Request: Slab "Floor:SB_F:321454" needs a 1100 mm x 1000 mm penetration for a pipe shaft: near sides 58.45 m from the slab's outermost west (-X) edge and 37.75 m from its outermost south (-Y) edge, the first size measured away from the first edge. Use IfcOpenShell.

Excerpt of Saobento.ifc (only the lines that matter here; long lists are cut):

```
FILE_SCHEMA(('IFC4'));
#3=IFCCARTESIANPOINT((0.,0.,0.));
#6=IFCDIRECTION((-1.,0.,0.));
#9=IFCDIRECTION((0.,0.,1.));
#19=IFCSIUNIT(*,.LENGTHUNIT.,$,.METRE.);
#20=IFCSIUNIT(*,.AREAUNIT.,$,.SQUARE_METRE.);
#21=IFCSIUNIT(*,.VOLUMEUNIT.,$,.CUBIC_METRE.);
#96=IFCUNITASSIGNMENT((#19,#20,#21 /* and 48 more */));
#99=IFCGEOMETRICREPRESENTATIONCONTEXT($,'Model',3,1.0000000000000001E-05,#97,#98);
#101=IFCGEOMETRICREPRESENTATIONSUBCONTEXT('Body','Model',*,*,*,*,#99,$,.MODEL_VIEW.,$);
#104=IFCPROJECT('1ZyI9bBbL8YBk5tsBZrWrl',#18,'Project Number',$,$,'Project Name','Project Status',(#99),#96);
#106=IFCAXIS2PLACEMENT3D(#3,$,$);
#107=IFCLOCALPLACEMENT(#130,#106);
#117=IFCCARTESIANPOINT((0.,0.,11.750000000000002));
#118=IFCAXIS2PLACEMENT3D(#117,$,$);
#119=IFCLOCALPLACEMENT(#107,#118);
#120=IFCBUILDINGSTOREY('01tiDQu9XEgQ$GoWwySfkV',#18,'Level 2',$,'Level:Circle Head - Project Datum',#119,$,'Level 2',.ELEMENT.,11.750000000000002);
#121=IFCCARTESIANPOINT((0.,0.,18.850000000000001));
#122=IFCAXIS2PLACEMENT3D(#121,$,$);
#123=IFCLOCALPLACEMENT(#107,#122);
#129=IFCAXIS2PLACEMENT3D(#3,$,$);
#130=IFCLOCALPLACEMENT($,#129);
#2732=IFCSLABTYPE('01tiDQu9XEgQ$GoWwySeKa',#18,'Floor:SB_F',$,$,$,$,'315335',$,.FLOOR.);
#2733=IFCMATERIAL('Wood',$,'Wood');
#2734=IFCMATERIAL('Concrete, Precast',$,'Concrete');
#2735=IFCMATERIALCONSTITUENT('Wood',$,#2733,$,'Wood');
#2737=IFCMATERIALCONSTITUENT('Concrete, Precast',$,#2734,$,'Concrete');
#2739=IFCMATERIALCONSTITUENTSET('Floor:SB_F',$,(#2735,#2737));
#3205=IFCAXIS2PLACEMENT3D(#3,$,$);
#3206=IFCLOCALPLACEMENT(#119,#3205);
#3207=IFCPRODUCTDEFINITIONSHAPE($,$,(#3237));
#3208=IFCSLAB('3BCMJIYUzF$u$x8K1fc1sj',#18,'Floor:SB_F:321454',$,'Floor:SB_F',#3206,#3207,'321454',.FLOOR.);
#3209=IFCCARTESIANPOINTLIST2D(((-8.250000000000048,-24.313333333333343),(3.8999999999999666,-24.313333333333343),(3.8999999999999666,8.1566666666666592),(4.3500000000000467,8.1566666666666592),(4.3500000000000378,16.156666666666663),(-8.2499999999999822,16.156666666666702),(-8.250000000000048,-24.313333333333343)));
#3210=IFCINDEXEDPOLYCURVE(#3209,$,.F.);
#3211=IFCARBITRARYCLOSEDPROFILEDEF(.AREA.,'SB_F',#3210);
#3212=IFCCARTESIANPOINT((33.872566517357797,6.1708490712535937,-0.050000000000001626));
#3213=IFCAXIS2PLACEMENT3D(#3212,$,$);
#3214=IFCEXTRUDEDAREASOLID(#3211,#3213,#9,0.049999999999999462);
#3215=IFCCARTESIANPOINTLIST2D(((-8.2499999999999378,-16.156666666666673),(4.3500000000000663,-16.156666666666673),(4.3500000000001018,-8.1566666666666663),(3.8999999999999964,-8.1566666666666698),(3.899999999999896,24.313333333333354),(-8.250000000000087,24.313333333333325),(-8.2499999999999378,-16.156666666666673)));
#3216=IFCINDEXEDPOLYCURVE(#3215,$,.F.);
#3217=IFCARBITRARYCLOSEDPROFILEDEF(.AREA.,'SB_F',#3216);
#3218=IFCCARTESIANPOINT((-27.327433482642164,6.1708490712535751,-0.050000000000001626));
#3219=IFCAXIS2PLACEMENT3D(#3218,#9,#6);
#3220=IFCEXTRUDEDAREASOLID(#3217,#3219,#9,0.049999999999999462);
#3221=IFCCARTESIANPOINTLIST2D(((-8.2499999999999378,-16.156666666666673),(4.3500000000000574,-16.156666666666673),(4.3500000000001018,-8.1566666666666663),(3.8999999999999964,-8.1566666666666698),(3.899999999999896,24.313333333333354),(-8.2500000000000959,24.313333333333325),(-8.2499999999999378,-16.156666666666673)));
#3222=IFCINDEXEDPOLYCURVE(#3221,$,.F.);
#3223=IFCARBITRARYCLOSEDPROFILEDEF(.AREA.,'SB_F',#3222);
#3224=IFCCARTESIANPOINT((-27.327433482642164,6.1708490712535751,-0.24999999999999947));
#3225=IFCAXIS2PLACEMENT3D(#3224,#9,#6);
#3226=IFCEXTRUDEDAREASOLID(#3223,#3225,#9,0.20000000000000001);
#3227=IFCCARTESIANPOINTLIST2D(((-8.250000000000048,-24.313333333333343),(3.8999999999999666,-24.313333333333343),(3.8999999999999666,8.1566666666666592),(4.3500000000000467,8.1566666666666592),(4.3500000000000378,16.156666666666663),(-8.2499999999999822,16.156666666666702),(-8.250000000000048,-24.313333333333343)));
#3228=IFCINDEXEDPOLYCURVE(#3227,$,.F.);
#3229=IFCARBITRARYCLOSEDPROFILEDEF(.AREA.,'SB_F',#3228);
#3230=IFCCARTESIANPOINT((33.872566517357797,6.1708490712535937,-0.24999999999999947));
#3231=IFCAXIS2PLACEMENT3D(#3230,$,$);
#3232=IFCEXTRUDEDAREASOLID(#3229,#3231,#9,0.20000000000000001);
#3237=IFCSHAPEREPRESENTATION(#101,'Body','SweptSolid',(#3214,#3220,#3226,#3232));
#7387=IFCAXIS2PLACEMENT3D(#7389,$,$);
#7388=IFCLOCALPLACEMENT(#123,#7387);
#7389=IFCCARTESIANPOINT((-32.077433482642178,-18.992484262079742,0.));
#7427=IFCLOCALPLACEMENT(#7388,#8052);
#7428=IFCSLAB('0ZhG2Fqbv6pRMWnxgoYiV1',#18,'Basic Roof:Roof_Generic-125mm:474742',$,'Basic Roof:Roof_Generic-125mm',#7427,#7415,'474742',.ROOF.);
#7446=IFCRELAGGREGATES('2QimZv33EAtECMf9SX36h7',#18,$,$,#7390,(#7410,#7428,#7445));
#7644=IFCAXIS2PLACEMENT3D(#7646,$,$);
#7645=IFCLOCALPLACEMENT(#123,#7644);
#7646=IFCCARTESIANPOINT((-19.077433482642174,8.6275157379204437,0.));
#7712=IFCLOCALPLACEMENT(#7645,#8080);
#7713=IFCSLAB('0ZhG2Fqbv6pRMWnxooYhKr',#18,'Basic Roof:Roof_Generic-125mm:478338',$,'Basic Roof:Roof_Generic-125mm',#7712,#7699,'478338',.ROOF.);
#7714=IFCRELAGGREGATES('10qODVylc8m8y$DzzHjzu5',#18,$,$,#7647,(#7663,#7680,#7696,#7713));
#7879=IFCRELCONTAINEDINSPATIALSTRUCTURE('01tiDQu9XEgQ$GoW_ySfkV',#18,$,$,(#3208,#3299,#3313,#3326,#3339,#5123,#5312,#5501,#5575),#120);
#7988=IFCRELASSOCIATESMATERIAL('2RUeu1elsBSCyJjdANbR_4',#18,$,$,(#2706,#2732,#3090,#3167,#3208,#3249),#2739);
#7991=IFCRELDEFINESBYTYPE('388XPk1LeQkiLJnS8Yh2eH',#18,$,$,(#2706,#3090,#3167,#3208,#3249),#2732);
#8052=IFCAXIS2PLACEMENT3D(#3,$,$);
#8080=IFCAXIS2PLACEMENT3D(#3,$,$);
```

```python
import numpy as np
import ifcopenshell
import ifcopenshell.api.feature
import ifcopenshell.api.geometry
import ifcopenshell.api.root
import ifcopenshell.geom
import ifcopenshell.util.placement
import ifcopenshell.util.representation
import ifcopenshell.util.shape
import ifcopenshell.util.unit

model = ifcopenshell.open("Saobento.ifc")
unit_scale = ifcopenshell.util.unit.calculate_unit_scale(model)
settings = ifcopenshell.geom.settings()


def volume(element):
    """Net volume in cubic metres, openings subtracted."""
    shape = ifcopenshell.geom.create_shape(settings, element)
    return ifcopenshell.util.shape.get_volume(shape.geometry)


slab = model.by_guid("3BCMJIYUzF$u$x8K1fc1sj")
before = volume(slab)

# Extent in the slab's own axes, in metres. The edges named are its -X and -Y sides.
slab_shape = ifcopenshell.geom.create_shape(settings, slab)
vertices = ifcopenshell.util.shape.get_vertices(slab_shape.geometry)
x_min, y_min, bottom = vertices.min(axis=0)
top = vertices[:, 2].max()

opening = ifcopenshell.api.root.create_entity(model, ifc_class="IfcOpeningElement", name="Pipe shaft opening", predefined_type="OPENING")
context = ifcopenshell.util.representation.get_context(model, "Model", "Body", "MODEL_VIEW")
width, depth = 1.1, 1
outline = [(0.0, 0.0), (width, 0.0), (width, depth), (0.0, depth), (0.0, 0.0)]
# Overshoot both faces by 50 mm so the cut is clean.
shape = ifcopenshell.api.geometry.add_slab_representation(
    model, context=context, depth=top - bottom + 0.1, polyline=outline
)
ifcopenshell.api.geometry.assign_representation(model, product=opening, representation=shape)

matrix = ifcopenshell.util.placement.get_local_placement(slab.ObjectPlacement)
matrix[:, 3] = matrix @ np.append(np.array([x_min + 58.45, y_min + 37.75, bottom - 0.05]) / unit_scale, 1.0)
ifcopenshell.api.geometry.edit_object_placement(model, product=opening, matrix=matrix, is_si=False)
ifcopenshell.api.feature.add_feature(model, feature=opening, element=slab)

after = volume(slab)

print(f"slab volume {before:.3f} -> {after:.3f} m3")

model.write("Saobento_edited.ifc")
```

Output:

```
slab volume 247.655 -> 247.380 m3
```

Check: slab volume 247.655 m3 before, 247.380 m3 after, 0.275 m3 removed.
